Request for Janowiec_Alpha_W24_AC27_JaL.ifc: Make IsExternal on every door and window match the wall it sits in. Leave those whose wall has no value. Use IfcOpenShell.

First a look at what the model holds.

```python
import ifcopenshell
import ifcopenshell.util.element

model = ifcopenshell.open("Janowiec_Alpha_W24_AC27_JaL.ifc")
print(model.schema)
seen = {}
for e in model.by_type("IfcDoor") + model.by_type("IfcWindow"):
    if not e.FillsVoids:
        continue
    host = e.FillsVoids[0].RelatingOpeningElement.VoidsElements[0].RelatingBuildingElement
    own = ifcopenshell.util.element.get_pset(e, f"Pset_{e.is_a()[3:].removesuffix('StandardCase')}Common", "IsExternal")
    wall = ifcopenshell.util.element.get_pset(host, "Pset_WallCommon", "IsExternal")
    seen[e.is_a(), own, wall] = seen.get((e.is_a(), own, wall), 0) + 1
for (cls, own, wall), count in sorted(seen.items(), key=str):
    print(count, cls, "IsExternal:", own, "| host wall:", wall)
```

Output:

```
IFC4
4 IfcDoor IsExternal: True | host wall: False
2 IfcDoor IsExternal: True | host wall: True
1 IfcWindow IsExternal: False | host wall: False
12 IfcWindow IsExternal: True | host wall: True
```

```python
import ifcopenshell
import ifcopenshell.api.pset
import ifcopenshell.util.element

model = ifcopenshell.open("Janowiec_Alpha_W24_AC27_JaL.ifc")

count = 0
for ifc_class, pset_name in (("IfcDoor", "Pset_DoorCommon"), ("IfcWindow", "Pset_WindowCommon")):
    for e in model.by_type(ifc_class):
        if not e.FillsVoids:
            continue
        host = e.FillsVoids[0].RelatingOpeningElement.VoidsElements[0].RelatingBuildingElement
        external = ifcopenshell.util.element.get_pset(host, "Pset_WallCommon", "IsExternal")
        if external is None or ifcopenshell.util.element.get_pset(e, pset_name, "IsExternal") == external:
            continue
        pset = ifcopenshell.api.pset.add_pset(model, product=e, name=pset_name)
        ifcopenshell.api.pset.edit_pset(model, pset=pset, properties={"IsExternal": external})
        count += 1

print(count, "updated")

model.write("Janowiec_Alpha_W24_AC27_JaL_updated.ifc")
```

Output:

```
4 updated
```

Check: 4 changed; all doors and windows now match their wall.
